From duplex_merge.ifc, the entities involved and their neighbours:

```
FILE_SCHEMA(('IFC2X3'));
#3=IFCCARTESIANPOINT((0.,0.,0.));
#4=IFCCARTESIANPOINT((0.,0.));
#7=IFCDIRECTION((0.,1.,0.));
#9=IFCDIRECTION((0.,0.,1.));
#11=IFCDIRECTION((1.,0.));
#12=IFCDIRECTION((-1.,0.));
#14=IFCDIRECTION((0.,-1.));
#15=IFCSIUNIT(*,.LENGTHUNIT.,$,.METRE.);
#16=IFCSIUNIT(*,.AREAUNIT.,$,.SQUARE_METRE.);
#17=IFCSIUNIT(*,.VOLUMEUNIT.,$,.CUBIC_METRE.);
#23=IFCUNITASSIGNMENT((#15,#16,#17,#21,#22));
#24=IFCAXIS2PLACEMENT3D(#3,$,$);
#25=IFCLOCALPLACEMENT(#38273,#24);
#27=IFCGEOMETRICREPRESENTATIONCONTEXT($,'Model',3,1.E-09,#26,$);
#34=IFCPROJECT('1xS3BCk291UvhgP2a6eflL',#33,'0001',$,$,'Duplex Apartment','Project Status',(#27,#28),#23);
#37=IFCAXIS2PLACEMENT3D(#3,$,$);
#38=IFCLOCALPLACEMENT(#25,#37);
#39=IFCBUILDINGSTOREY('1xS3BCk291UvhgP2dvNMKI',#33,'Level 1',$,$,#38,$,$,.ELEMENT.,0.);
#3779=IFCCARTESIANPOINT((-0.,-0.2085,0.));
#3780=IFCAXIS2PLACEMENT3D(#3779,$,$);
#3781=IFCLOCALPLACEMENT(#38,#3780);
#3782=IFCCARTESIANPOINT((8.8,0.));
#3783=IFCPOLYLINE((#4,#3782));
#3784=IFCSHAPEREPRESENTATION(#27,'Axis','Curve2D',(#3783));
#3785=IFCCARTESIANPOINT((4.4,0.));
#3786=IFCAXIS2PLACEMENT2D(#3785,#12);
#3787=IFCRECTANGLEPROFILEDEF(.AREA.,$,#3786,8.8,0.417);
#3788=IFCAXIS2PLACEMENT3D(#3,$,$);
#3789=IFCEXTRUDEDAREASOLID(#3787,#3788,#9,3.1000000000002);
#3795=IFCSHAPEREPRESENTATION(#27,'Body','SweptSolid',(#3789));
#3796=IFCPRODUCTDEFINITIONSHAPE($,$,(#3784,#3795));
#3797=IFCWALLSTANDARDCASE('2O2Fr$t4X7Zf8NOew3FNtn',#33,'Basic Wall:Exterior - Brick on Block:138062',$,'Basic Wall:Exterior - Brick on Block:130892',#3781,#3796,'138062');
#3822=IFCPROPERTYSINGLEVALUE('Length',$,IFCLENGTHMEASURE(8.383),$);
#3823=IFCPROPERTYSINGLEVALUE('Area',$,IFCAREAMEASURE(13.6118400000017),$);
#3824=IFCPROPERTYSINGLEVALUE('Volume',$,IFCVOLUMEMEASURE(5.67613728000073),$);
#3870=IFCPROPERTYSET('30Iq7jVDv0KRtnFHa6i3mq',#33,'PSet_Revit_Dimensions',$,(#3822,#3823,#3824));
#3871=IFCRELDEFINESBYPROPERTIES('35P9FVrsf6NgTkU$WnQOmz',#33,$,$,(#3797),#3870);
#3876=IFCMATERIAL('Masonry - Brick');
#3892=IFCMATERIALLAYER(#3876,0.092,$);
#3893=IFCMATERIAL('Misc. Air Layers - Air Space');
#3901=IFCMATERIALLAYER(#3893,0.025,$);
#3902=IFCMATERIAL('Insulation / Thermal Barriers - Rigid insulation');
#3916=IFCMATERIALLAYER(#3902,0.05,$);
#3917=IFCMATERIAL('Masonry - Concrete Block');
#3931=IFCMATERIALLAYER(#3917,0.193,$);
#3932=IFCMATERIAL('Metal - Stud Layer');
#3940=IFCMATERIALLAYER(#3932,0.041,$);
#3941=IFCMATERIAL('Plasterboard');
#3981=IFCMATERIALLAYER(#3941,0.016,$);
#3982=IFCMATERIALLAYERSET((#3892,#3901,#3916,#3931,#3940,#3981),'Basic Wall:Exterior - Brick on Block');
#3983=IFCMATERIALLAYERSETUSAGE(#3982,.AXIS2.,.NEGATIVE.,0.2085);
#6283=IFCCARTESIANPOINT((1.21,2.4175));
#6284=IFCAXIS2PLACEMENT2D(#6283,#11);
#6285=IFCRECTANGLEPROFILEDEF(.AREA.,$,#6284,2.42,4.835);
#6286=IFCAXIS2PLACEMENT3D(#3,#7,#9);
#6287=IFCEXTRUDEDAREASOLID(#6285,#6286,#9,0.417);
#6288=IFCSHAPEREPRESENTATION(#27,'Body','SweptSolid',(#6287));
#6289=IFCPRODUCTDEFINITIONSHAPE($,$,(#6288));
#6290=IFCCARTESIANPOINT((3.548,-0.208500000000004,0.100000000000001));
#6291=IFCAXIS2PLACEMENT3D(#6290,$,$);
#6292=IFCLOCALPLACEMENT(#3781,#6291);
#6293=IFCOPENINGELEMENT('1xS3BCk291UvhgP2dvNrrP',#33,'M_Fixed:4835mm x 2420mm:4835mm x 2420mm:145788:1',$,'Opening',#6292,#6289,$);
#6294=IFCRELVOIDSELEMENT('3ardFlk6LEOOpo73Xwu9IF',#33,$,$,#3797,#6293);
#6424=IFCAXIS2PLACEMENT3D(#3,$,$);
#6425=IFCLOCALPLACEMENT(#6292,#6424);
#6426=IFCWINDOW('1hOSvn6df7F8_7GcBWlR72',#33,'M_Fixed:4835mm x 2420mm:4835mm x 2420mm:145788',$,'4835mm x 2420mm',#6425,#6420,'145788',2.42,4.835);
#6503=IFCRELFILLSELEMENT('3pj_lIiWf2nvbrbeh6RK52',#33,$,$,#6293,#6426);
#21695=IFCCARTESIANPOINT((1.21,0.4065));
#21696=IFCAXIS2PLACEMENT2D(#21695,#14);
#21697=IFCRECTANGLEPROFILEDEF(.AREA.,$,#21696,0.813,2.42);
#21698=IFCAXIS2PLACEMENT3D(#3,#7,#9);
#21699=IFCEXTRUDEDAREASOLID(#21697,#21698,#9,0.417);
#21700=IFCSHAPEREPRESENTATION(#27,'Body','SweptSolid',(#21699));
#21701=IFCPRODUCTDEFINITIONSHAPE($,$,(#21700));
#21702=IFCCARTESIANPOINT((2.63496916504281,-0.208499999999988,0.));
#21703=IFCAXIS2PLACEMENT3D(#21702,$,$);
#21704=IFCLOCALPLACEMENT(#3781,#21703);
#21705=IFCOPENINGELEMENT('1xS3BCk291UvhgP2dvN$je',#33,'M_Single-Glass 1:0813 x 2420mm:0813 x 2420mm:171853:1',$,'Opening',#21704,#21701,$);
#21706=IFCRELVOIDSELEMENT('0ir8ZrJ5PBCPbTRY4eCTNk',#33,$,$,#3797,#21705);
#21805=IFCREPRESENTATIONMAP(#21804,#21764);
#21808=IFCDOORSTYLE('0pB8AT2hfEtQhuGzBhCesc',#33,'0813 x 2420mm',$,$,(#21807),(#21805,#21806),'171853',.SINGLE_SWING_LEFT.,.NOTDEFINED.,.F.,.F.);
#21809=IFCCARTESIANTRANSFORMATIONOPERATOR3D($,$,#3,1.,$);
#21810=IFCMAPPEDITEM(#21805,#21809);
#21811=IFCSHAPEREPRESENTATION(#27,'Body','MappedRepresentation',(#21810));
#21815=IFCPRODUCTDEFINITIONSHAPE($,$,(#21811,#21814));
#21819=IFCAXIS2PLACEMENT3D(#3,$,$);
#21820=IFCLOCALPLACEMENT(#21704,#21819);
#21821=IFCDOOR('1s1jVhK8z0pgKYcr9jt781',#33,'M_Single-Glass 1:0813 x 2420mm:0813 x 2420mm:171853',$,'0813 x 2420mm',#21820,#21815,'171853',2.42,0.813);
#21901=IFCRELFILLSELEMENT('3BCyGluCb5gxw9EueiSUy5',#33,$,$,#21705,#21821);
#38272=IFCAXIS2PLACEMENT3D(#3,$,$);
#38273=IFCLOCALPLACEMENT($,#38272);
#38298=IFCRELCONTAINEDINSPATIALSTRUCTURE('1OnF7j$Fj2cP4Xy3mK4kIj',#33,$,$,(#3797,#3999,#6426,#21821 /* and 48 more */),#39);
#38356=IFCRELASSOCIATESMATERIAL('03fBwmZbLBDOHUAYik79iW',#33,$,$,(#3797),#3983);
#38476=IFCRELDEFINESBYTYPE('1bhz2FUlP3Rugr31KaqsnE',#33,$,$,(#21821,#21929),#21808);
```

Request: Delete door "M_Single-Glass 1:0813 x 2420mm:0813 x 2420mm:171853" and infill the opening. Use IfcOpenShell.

```python
import ifcopenshell
import ifcopenshell.api.feature
import ifcopenshell.api.pset
import ifcopenshell.api.root
import ifcopenshell.geom
import ifcopenshell.util.element
import ifcopenshell.util.shape
import ifcopenshell.util.unit

model = ifcopenshell.open("duplex_merge.ifc")
area_scale = ifcopenshell.util.unit.calculate_unit_scale(model, "AREAUNIT")
volume_scale = ifcopenshell.util.unit.calculate_unit_scale(model, "VOLUMEUNIT")
settings = ifcopenshell.geom.settings()


def volume(element):
    """Net volume in cubic metres, openings subtracted."""
    shape = ifcopenshell.geom.create_shape(settings, element)
    return ifcopenshell.util.shape.get_volume(shape.geometry)


door = model.by_id(21821)
opening = door.FillsVoids[0].RelatingOpeningElement
wall = opening.VoidsElements[0].RelatingBuildingElement
before = volume(wall)

ifcopenshell.api.root.remove_product(model, product=door)
ifcopenshell.api.feature.remove_feature(model, feature=opening)

after = volume(wall)
thickness = 0.417  # wall thickness in metres

# Update the wall's stored quantities.
pset = model.by_id(ifcopenshell.util.element.get_pset(wall, "PSet_Revit_Dimensions", should_inherit=False)["id"])
ifcopenshell.api.pset.edit_pset(model, pset=pset, properties={
    "Area": model.create_entity("IfcAreaMeasure", after / thickness / area_scale),
    "Volume": model.create_entity("IfcVolumeMeasure", after / volume_scale),
})

print(f"wall volume {before:.3f} -> {after:.3f} m3")

model.write("duplex_merge_edited.ifc")
```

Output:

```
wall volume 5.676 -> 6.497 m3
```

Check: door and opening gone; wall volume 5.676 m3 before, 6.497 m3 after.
